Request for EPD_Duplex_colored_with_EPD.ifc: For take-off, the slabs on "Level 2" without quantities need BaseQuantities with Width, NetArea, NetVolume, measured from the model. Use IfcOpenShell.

First a look at what the model holds.

```python
import ifcopenshell
import ifcopenshell.util.element
import ifcopenshell.util.unit

model = ifcopenshell.open("EPD_Duplex_colored_with_EPD.ifc")
print(model.schema)
for unit_type in ("LENGTHUNIT", "AREAUNIT", "VOLUMEUNIT"):
    print(unit_type, ifcopenshell.util.unit.calculate_unit_scale(model, unit_type))
storey = next(s for s in model.by_type("IfcBuildingStorey") if s.Name == "Level 2")
slabs = [e for e in ifcopenshell.util.element.get_decomposition(storey) if e.is_a("IfcSlab")]
for e in sorted(slabs, key=lambda e: e.id()):
    print(e.id(), e.is_a(), e.Name, list(ifcopenshell.util.element.get_psets(e, qtos_only=True)), sep=" | ")
```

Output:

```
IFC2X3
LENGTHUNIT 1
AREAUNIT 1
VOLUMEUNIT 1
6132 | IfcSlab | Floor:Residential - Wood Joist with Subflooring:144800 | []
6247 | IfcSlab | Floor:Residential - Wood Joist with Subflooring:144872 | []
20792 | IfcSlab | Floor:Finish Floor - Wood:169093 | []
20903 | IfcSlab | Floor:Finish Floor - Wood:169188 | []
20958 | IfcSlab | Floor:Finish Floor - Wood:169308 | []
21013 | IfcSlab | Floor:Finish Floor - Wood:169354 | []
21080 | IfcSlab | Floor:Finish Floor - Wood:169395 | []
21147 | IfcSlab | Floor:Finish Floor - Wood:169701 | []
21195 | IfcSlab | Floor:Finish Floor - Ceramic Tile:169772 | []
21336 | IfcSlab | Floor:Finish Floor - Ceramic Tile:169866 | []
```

```python
import ifcopenshell
import ifcopenshell.api.pset
import ifcopenshell.geom
import ifcopenshell.util.element
import ifcopenshell.util.shape
import ifcopenshell.util.unit

model = ifcopenshell.open("EPD_Duplex_colored_with_EPD.ifc")
unit_scale = ifcopenshell.util.unit.calculate_unit_scale(model)
area_scale = ifcopenshell.util.unit.calculate_unit_scale(model, "AREAUNIT")
volume_scale = ifcopenshell.util.unit.calculate_unit_scale(model, "VOLUMEUNIT")
settings = ifcopenshell.geom.settings()

storey = next(s for s in model.by_type("IfcBuildingStorey") if s.Name == "Level 2")
slabs = [e for e in ifcopenshell.util.element.get_decomposition(storey) if e.is_a("IfcSlab")]

for e in sorted(slabs, key=lambda e: e.id()):
    if ifcopenshell.util.element.get_psets(e, qtos_only=True, should_inherit=False):
        continue
    # Geometry comes back in metres, in the element's own axes.
    shape = ifcopenshell.geom.create_shape(settings, e)
    values = {
        "Width": ifcopenshell.util.shape.get_z(shape.geometry) / unit_scale,
        "NetArea": ifcopenshell.util.shape.get_footprint_area(shape.geometry) / area_scale,
        "NetVolume": ifcopenshell.util.shape.get_volume(shape.geometry) / volume_scale,
    }
    qto = ifcopenshell.api.pset.add_qto(model, product=e, name="BaseQuantities")
    ifcopenshell.api.pset.edit_qto(model, qto=qto, properties=values)
    print(e.id(), {k: round(v, 3) for k, v in values.items()})

model.write("EPD_Duplex_colored_with_EPD_v2.ifc")
```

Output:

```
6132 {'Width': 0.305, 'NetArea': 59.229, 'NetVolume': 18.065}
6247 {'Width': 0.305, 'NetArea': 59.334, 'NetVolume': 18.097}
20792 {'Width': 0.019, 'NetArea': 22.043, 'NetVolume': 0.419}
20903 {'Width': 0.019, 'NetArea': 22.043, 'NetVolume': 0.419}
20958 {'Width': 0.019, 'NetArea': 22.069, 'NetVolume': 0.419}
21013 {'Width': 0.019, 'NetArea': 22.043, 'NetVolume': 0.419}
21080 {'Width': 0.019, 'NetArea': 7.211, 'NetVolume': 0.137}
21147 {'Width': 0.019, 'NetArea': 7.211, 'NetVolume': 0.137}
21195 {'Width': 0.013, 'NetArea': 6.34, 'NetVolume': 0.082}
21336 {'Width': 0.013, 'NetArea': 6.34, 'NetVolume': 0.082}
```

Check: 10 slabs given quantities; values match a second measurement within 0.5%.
